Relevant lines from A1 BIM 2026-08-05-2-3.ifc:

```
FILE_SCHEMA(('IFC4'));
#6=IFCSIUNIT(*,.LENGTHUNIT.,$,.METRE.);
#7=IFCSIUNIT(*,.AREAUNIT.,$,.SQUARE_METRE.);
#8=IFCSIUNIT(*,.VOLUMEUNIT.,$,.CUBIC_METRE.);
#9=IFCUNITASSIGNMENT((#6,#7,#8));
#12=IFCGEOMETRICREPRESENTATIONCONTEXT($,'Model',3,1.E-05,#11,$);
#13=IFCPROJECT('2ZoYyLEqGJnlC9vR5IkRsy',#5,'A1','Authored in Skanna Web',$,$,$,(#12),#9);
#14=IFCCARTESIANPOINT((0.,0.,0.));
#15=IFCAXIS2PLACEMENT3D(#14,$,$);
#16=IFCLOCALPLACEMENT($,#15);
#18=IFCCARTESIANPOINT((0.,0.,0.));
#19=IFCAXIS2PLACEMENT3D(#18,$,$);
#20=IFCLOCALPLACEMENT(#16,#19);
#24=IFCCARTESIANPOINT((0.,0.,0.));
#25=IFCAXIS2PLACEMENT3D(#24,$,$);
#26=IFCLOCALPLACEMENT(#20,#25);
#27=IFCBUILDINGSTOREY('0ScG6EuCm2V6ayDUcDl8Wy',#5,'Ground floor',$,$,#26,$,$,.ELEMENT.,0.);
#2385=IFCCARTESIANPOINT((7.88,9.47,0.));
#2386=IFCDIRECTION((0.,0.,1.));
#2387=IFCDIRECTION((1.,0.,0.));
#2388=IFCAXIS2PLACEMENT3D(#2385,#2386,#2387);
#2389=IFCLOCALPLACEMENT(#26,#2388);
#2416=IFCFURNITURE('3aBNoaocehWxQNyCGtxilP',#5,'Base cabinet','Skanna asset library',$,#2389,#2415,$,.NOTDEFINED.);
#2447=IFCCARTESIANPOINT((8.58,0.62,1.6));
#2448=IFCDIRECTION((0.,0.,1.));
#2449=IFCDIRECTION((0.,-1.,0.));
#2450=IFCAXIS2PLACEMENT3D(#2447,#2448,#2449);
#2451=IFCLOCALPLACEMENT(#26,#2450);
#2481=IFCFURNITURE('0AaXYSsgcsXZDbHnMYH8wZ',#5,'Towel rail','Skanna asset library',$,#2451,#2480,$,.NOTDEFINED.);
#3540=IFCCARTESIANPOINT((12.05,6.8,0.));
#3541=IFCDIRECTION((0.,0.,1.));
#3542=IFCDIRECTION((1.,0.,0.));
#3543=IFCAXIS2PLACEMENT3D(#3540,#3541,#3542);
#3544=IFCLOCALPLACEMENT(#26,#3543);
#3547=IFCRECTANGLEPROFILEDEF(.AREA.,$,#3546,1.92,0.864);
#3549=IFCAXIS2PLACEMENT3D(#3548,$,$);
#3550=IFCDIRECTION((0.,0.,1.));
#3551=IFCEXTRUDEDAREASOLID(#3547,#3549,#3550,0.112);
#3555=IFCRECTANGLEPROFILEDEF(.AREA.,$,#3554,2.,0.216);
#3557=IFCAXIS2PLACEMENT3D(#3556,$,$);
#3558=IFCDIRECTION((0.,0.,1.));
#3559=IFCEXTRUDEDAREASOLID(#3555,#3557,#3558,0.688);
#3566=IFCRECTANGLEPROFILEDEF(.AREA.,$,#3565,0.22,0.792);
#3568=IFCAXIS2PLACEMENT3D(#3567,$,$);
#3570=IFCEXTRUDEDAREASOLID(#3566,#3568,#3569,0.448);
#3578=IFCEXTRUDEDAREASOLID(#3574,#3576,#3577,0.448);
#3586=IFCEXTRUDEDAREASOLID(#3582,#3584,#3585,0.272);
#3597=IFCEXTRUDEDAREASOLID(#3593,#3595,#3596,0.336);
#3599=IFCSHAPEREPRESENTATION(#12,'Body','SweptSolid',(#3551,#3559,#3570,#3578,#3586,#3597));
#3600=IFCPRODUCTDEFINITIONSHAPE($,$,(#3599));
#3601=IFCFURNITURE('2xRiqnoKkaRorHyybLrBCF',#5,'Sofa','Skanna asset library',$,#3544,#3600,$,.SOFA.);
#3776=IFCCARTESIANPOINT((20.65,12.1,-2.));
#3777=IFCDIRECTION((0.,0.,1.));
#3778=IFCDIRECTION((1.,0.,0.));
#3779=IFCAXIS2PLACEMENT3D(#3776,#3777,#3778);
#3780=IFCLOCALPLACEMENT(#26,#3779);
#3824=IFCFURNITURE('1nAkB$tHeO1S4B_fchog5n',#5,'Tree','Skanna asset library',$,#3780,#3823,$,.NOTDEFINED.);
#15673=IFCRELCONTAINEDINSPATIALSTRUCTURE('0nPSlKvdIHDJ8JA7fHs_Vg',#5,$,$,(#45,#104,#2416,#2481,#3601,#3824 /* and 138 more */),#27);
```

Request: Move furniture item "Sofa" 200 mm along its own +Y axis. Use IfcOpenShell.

```python
import ifcopenshell
import ifcopenshell.api.geometry
import ifcopenshell.util.placement

model = ifcopenshell.open("A1 BIM 2026-08-05-2-3.ifc")

item = model.by_guid("2xRiqnoKkaRorHyybLrBCF")
matrix = ifcopenshell.util.placement.get_local_placement(item.ObjectPlacement)
matrix[:3, 3] += matrix[:3, 1] * 0.2
ifcopenshell.api.geometry.edit_object_placement(model, product=item, matrix=matrix, is_si=False)

print(ifcopenshell.util.placement.get_local_placement(item.ObjectPlacement).round(3) + 0.0)

model.write("A1 BIM 2026-08-05-2-3_updated.ifc")
```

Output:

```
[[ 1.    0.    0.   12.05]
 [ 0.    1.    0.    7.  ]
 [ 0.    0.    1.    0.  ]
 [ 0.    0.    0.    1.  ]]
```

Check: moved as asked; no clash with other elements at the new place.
